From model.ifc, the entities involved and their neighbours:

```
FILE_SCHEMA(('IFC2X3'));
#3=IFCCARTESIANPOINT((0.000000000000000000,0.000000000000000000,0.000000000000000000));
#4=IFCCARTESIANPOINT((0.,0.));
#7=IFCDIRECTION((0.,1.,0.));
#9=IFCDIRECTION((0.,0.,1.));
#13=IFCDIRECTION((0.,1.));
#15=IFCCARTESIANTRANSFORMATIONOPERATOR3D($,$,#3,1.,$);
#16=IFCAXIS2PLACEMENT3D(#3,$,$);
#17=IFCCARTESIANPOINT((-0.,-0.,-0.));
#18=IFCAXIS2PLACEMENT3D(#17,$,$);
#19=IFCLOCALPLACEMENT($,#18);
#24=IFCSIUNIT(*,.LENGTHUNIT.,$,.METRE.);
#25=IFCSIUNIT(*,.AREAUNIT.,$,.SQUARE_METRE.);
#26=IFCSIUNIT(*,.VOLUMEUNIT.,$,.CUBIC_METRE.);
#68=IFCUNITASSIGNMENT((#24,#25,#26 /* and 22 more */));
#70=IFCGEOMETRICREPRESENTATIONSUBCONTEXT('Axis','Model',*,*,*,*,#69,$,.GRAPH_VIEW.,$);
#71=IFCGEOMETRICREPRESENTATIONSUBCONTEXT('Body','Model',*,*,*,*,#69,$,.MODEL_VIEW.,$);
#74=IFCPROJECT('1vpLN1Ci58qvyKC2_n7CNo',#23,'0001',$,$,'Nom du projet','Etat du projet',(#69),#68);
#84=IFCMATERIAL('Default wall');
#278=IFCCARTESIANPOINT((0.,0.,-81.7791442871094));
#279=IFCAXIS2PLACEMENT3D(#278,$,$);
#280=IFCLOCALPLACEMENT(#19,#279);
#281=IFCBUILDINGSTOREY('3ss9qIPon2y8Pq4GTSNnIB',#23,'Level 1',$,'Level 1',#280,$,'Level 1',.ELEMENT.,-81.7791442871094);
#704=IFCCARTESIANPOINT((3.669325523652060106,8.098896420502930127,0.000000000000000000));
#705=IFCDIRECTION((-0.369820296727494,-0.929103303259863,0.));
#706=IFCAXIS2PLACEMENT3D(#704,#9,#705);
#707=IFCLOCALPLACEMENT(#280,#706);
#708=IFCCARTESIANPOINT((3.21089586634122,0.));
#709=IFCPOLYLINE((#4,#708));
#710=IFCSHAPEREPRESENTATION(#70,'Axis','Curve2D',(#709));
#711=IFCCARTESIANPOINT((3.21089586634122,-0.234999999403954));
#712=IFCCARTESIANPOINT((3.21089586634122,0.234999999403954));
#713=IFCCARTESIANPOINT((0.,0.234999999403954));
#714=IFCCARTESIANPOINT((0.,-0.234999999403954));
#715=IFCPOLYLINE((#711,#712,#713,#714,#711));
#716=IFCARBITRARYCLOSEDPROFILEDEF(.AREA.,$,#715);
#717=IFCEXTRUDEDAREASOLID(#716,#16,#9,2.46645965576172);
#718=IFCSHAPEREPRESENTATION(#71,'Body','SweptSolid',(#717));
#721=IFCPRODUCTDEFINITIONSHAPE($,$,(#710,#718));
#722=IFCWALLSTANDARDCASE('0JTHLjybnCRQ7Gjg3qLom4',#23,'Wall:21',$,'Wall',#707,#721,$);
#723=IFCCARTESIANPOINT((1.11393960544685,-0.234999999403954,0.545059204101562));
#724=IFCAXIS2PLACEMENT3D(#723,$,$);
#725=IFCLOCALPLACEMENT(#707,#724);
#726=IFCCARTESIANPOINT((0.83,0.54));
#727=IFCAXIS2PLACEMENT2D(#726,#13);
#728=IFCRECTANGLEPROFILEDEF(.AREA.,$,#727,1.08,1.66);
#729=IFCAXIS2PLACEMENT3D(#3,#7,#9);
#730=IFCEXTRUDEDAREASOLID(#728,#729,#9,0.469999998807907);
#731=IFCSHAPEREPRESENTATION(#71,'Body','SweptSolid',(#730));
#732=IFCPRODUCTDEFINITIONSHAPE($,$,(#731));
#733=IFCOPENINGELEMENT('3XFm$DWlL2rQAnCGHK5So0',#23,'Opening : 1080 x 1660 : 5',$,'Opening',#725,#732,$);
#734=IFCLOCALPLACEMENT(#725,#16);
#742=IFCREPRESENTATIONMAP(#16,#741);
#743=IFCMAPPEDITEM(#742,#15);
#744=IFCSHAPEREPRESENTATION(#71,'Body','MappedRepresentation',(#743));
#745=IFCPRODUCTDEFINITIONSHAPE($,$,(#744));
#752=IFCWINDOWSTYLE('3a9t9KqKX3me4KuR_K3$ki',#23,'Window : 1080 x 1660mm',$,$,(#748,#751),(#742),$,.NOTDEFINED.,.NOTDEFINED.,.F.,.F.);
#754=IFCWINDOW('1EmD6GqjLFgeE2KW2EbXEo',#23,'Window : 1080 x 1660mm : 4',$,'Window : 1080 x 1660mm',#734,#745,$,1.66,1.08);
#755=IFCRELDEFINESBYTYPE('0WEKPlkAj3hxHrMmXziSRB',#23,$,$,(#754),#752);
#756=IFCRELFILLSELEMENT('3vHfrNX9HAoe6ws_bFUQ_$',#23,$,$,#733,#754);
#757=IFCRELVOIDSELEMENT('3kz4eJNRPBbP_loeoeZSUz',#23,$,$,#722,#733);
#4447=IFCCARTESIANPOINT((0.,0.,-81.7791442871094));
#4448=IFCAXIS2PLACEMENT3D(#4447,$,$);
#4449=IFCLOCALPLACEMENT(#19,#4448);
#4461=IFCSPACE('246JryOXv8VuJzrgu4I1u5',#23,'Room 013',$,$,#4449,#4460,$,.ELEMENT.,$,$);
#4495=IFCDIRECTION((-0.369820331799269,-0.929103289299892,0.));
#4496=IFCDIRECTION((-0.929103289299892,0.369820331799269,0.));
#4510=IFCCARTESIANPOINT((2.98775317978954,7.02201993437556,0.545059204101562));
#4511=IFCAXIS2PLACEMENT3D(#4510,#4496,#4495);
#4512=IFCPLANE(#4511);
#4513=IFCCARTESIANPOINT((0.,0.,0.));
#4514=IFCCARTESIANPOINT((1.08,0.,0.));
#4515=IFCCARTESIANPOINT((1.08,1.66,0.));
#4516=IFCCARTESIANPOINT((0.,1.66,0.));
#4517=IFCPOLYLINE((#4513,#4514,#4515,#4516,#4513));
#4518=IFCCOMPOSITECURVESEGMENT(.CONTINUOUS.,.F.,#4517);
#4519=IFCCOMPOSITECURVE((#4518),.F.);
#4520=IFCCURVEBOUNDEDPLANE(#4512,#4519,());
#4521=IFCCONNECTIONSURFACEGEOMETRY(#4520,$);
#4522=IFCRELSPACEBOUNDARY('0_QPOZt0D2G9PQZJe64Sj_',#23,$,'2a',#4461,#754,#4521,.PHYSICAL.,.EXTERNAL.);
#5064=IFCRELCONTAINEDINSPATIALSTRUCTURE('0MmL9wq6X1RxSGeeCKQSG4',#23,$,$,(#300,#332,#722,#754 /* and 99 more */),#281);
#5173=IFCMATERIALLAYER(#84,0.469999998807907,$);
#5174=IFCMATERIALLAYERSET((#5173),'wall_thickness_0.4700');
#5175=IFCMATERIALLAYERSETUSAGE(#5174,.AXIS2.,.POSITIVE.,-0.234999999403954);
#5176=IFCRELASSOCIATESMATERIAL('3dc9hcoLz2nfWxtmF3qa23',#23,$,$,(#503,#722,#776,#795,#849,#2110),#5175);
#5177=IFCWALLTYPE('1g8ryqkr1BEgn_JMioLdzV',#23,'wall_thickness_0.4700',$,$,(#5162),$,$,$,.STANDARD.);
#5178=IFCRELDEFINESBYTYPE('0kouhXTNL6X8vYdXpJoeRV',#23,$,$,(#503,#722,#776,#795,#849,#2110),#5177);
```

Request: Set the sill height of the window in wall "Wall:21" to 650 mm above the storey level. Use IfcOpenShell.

```python
import numpy as np
import ifcopenshell
import ifcopenshell.api.geometry
import ifcopenshell.geom
import ifcopenshell.util.element
import ifcopenshell.util.placement
import ifcopenshell.util.shape
import ifcopenshell.util.unit

model = ifcopenshell.open("model.ifc")
unit_scale = ifcopenshell.util.unit.calculate_unit_scale(model)

window = model.by_id(754)
opening = window.FillsVoids[0].RelatingOpeningElement
storey = ifcopenshell.util.element.get_container(window, ifc_class="IfcBuildingStorey")
level = ifcopenshell.util.placement.get_local_placement(storey.ObjectPlacement)[2, 3]

# The opening's origin need not be at the sill, so measure its lowest point.
shape = ifcopenshell.geom.create_shape(ifcopenshell.geom.settings(), opening)
bottom = ifcopenshell.util.shape.get_shape_bottom_elevation(shape, shape.geometry) / unit_scale
dz = level + 0.65 / unit_scale - bottom

shift = np.array([0.0, 0.0, dz])
# The window is placed relative to its opening, so it follows when the opening moves.
matrix = ifcopenshell.util.placement.get_local_placement(opening.ObjectPlacement)
matrix[:3, 3] += shift
ifcopenshell.api.geometry.edit_object_placement(
    model, product=opening, matrix=matrix, is_si=False, should_transform_children=True
)

# Space boundary surfaces are stored in each space's coordinates; move them too.
for rel in window.ProvidesBoundaries:
    if not rel.ConnectionGeometry:
        continue
    surface = rel.ConnectionGeometry.SurfaceOnRelatingElement.BasisSurface
    space_matrix = ifcopenshell.util.placement.get_local_placement(rel.RelatingSpace.ObjectPlacement)
    point = np.array(surface.Position.Location.Coordinates) + space_matrix[:3, :3].T @ shift
    surface.Position = model.createIfcAxis2Placement3D(
        model.createIfcCartesianPoint(point.tolist()), surface.Position.Axis, surface.Position.RefDirection
    )

print(f"moved by {dz * unit_scale:+.3f} m")

model.write("model-out.ifc")
```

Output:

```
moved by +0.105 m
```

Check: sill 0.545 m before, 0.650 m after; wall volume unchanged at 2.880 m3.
